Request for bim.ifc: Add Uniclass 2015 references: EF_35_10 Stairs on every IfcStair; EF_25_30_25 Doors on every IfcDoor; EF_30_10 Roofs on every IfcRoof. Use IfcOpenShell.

First a look at what the model holds.

```python
import ifcopenshell

model = ifcopenshell.open("bim.ifc")
print(model.schema)
print("classifications:", [c.Name for c in model.by_type("IfcClassification")])
for ifc_class in ("IfcDoor", "IfcRoof", "IfcStair", "IfcWall", "IfcWindow"):
    print(ifc_class, len(model.by_type(ifc_class)))
```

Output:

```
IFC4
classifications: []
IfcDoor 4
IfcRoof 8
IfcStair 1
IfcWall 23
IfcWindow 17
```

```python
import ifcopenshell
import ifcopenshell.api.classification

model = ifcopenshell.open("bim.ifc")

system = ifcopenshell.api.classification.add_classification(model, classification="Uniclass 2015")

codes = {
    "IfcStair": ("EF_35_10", "Stairs"),
    "IfcDoor": ("EF_25_30_25", "Doors"),
    "IfcRoof": ("EF_30_10", "Roofs"),
}
for ifc_class, (code, name) in codes.items():
    products = model.by_type(ifc_class)
    ifcopenshell.api.classification.add_reference(
        model, products=products, classification=system, identification=code, name=name
    )
    print(code, len(products))

model.write("bim-out.ifc")
```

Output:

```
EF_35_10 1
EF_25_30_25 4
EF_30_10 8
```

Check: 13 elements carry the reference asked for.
